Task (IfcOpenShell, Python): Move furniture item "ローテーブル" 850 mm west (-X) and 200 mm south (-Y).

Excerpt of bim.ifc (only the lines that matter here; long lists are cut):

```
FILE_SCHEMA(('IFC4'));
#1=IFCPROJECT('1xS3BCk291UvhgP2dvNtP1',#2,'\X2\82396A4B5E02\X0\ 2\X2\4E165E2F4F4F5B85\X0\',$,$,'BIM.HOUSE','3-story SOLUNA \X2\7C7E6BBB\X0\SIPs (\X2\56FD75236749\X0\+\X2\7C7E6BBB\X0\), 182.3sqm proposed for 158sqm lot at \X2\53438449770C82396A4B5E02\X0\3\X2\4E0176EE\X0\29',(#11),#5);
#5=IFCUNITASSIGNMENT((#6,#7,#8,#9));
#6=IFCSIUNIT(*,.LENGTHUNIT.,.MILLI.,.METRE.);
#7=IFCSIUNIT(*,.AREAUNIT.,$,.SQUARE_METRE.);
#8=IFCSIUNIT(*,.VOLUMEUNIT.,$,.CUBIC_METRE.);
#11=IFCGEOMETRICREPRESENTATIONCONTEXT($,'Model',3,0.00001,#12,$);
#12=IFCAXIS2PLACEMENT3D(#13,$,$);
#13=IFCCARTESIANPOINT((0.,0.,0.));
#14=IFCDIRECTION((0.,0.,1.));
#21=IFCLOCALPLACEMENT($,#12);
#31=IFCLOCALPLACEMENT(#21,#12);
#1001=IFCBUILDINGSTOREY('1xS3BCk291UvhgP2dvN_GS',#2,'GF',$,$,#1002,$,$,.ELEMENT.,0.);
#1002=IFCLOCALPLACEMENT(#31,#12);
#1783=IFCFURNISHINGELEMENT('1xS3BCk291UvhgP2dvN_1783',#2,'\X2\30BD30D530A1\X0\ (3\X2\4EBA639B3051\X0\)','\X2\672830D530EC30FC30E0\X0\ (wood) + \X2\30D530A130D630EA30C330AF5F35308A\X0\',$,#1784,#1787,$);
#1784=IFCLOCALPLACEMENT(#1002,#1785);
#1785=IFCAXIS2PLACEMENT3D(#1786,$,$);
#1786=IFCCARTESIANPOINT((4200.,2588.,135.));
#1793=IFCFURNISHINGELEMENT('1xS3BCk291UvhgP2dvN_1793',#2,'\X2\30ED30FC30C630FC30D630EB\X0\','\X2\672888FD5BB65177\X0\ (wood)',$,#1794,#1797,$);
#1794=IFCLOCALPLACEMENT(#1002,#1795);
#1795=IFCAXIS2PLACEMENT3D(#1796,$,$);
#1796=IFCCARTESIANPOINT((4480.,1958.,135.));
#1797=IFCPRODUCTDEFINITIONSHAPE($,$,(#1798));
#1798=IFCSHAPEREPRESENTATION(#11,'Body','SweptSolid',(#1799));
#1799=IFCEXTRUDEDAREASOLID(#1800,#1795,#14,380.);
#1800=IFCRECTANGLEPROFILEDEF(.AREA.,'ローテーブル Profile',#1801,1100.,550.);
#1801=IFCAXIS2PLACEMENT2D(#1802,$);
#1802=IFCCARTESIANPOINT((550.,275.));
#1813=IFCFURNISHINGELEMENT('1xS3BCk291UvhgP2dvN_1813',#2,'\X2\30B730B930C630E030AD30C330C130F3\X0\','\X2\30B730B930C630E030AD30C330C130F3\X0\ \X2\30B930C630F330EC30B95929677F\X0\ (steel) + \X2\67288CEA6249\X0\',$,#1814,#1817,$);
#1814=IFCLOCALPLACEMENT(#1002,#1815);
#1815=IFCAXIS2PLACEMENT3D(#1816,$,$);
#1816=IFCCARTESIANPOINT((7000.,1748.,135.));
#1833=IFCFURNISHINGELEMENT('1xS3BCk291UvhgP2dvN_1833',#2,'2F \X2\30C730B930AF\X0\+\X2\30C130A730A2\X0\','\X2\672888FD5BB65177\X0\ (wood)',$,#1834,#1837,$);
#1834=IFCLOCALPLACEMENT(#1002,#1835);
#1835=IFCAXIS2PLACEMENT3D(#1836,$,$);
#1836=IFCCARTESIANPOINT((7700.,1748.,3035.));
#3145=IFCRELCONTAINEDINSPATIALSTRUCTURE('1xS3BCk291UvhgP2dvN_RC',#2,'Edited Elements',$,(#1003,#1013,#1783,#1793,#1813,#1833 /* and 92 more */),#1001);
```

```python
import ifcopenshell
import ifcopenshell.api.geometry
import ifcopenshell.util.placement

model = ifcopenshell.open("bim.ifc")

item = model.by_guid("1xS3BCk291UvhgP2dvN_1793")
matrix = ifcopenshell.util.placement.get_local_placement(item.ObjectPlacement)
matrix[0, 3] -= 850.0
matrix[1, 3] -= 200.0
ifcopenshell.api.geometry.edit_object_placement(model, product=item, matrix=matrix, is_si=False)

print(ifcopenshell.util.placement.get_local_placement(item.ObjectPlacement).round(3) + 0.0)

model.write("bim_updated.ifc")
```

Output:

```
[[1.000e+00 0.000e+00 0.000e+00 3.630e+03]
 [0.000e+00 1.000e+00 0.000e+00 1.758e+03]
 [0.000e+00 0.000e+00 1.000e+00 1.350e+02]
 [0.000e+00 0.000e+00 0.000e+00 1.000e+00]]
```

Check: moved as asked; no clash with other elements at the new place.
